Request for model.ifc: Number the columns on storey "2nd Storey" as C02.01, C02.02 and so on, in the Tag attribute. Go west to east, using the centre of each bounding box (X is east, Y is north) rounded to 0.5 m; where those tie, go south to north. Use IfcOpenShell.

First a look at what the model holds.

```python
import ifcopenshell
import ifcopenshell.util.element
import ifcopenshell.util.placement

model = ifcopenshell.open("model.ifc")
print(model.schema)
storey = next(s for s in model.by_type("IfcBuildingStorey") if s.Name == "2nd Storey")
columns = [e for e in ifcopenshell.util.element.get_decomposition(storey) if e.is_a("IfcColumn")]
for e in sorted(columns, key=lambda e: e.id()):
    origin = ifcopenshell.util.placement.get_local_placement(e.ObjectPlacement)[:3, 3]
    print(e.id(), e.Tag, e.Name, origin.round(2) + 0.0, sep=" | ")
```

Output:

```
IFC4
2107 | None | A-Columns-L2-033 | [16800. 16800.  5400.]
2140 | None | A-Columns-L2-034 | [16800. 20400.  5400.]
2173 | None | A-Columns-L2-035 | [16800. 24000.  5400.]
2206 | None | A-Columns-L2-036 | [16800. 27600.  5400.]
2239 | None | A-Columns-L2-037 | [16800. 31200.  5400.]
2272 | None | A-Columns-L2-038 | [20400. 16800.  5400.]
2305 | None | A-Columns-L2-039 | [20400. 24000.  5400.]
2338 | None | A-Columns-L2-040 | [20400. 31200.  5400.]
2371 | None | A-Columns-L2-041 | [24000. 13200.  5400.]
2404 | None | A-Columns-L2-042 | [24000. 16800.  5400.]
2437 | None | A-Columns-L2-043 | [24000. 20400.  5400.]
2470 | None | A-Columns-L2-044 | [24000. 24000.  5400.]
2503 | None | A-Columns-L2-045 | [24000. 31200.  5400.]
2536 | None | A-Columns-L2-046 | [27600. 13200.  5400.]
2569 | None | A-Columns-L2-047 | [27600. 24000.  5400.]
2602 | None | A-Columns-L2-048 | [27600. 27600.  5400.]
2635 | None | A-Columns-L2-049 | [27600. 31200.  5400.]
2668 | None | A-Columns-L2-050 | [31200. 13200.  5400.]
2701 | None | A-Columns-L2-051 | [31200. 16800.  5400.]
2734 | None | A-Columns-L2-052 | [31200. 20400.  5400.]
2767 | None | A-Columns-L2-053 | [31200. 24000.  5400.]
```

```python
import ifcopenshell
import ifcopenshell.geom
import ifcopenshell.util.element
import ifcopenshell.util.shape

model = ifcopenshell.open("model.ifc")
settings = ifcopenshell.geom.settings()
settings.set("use-world-coords", True)


def centre(element):
    shape = ifcopenshell.geom.create_shape(settings, element)
    return ifcopenshell.util.shape.get_bbox_centroid(shape.geometry)


storey = next(s for s in model.by_type("IfcBuildingStorey") if s.Name == "2nd Storey")
columns = [e for e in ifcopenshell.util.element.get_decomposition(storey) if e.is_a("IfcColumn")]

# Insertion points can sit at a corner or the storey origin, so sort by the geometry (in metres).
centres = {e: centre(e) for e in columns}
columns.sort(key=lambda e: (round(centres[e][0] / 0.5), centres[e][1]))

for i, e in enumerate(columns, start=1):
    number = f"C02.{i:02d}"
    e.Tag = number
    print(e.id(), number)

model.write("model-out.ifc")
```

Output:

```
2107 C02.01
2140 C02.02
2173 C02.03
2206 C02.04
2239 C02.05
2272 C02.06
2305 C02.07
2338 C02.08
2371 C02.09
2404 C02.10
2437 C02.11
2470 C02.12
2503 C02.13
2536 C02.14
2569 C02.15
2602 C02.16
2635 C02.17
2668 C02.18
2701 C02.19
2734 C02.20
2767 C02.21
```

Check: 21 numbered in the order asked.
